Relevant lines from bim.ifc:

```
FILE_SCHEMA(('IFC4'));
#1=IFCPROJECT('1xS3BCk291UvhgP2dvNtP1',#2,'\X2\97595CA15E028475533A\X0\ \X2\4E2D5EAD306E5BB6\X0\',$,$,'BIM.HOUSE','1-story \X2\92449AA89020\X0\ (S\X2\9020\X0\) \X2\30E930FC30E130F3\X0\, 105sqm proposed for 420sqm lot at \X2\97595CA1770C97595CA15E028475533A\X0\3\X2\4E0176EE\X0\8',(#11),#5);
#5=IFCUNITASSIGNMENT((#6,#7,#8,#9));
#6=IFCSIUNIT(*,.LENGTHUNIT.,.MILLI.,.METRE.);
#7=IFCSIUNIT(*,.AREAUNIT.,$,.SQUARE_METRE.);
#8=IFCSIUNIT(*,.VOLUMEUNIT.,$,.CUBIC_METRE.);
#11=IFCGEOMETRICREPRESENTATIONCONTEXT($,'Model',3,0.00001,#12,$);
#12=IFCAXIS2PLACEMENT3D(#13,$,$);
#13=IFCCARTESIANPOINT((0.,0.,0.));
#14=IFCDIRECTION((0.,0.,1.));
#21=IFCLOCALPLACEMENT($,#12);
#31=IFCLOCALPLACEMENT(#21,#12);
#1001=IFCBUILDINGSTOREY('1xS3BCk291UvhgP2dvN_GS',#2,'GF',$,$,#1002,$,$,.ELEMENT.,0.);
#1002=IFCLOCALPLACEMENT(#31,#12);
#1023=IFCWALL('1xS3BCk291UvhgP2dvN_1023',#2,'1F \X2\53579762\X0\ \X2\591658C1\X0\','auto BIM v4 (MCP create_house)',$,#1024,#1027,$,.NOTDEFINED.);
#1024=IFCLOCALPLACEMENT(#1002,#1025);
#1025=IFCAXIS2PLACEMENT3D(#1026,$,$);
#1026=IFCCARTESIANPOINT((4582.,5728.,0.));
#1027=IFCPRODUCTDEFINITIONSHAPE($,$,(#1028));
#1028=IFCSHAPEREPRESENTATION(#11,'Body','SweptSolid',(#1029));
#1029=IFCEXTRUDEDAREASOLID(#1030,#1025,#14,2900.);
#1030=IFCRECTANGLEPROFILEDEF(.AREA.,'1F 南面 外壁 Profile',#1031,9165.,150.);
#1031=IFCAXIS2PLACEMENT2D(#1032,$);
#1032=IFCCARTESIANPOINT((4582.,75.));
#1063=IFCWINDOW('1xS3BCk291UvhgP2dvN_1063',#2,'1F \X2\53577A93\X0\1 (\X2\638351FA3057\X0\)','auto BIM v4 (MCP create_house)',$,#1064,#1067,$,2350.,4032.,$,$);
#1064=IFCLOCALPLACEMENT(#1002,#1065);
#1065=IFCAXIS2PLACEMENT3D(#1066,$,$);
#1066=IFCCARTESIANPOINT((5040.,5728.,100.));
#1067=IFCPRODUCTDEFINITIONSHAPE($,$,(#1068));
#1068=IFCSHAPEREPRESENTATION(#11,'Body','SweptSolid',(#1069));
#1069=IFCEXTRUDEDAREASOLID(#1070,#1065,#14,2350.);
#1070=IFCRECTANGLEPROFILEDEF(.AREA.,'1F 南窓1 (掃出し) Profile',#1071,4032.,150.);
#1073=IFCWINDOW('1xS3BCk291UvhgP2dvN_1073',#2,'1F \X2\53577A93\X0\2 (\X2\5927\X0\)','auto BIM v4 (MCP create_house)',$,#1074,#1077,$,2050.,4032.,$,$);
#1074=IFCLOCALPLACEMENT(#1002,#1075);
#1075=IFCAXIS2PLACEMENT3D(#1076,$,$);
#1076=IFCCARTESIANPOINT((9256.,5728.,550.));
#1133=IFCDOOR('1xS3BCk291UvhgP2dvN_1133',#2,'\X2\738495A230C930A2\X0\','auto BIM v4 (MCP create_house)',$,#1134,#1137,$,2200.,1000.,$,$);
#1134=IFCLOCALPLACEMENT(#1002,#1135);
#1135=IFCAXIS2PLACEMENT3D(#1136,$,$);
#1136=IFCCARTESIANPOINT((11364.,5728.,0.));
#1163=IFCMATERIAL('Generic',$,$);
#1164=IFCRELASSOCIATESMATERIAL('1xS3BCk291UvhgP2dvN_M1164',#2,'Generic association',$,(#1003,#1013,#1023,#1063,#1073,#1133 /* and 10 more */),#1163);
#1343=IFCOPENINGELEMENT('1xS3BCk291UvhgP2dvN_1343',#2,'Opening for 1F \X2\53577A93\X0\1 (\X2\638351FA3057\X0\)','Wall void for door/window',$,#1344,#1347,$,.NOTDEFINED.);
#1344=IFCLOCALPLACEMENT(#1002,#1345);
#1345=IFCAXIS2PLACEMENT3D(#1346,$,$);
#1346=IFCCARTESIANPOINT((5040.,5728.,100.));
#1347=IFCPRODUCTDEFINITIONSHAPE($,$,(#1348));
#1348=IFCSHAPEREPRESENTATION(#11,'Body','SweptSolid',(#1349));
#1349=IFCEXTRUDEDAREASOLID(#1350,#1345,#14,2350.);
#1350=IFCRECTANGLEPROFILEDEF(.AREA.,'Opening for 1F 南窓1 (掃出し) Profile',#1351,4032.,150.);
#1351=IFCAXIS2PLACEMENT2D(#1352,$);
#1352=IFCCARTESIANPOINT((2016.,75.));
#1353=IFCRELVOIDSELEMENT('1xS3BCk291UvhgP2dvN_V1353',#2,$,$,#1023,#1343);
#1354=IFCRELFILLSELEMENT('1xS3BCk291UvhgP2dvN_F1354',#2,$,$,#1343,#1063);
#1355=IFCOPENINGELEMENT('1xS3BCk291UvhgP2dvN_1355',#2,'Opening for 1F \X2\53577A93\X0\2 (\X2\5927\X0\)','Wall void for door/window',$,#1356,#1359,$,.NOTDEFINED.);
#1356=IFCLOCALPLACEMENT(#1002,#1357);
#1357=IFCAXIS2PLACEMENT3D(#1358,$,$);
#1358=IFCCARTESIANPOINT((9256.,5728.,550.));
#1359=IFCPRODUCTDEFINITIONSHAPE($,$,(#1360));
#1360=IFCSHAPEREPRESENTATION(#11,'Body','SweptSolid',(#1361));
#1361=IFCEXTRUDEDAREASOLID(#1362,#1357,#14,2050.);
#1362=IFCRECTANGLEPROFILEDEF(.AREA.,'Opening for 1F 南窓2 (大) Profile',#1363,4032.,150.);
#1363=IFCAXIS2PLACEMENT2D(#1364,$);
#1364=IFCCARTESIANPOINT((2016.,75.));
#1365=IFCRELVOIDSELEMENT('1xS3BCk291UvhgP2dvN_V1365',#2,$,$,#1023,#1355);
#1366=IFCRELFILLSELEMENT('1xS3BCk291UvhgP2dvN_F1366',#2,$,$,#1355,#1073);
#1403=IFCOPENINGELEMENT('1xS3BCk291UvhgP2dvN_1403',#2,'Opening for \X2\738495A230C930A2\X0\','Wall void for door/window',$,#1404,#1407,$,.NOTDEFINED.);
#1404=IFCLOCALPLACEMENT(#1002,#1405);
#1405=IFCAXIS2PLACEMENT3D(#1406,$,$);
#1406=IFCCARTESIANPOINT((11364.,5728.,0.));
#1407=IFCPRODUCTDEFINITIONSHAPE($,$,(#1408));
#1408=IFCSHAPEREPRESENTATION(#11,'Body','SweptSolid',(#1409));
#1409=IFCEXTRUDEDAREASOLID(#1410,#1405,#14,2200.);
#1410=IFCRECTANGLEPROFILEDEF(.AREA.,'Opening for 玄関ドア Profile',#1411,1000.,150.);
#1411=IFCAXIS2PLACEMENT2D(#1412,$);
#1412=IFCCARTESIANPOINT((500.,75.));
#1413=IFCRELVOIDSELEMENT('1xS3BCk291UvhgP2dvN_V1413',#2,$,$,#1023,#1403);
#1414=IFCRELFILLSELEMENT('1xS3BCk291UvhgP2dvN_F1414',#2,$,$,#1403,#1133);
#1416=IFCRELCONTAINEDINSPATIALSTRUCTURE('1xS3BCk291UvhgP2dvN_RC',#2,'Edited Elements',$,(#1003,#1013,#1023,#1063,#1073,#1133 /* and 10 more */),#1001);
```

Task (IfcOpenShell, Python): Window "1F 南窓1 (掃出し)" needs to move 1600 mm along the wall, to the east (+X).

```python
import ifcopenshell
import ifcopenshell.api.geometry
import ifcopenshell.util.placement
import ifcopenshell.util.unit

model = ifcopenshell.open("bim.ifc")
unit_scale = ifcopenshell.util.unit.calculate_unit_scale(model)

window = model.by_guid("1xS3BCk291UvhgP2dvN_1063")
opening = window.FillsVoids[0].RelatingOpeningElement
wall = opening.VoidsElements[0].RelatingBuildingElement

wall_matrix = ifcopenshell.util.placement.get_local_placement(wall.ObjectPlacement)
shift = wall_matrix[:3, 0] * 1.6 / unit_scale
before = ifcopenshell.util.placement.get_local_placement(window.ObjectPlacement)[:3, 3].copy()

# The window is not placed relative to its opening, so move both.
for product in (opening, window):
    matrix = ifcopenshell.util.placement.get_local_placement(product.ObjectPlacement)
    matrix[:3, 3] += shift
    ifcopenshell.api.geometry.edit_object_placement(model, product=product, matrix=matrix, is_si=False)

after = ifcopenshell.util.placement.get_local_placement(window.ObjectPlacement)[:3, 3]
print("window moved by", (after - before).round(3) + 0.0)

model.write("bim_rev.ifc")
```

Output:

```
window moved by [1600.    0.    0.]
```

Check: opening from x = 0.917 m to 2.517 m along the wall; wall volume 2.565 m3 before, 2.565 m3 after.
